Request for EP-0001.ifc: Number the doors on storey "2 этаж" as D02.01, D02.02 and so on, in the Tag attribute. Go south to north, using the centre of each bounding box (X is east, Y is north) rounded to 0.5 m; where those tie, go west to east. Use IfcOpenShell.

First a look at what the model holds.

```python
import ifcopenshell
import ifcopenshell.util.element
import ifcopenshell.util.placement

model = ifcopenshell.open("EP-0001.ifc")
print(model.schema)
storey = next(s for s in model.by_type("IfcBuildingStorey") if s.Name == "2 этаж")
doors = [e for e in ifcopenshell.util.element.get_decomposition(storey) if e.is_a("IfcDoor")]
for e in sorted(doors, key=lambda e: e.id()):
    origin = ifcopenshell.util.placement.get_local_placement(e.ObjectPlacement)[:3, 3]
    print(e.id(), e.Tag, e.Name, origin.round(2) + 0.0, sep=" | ")
```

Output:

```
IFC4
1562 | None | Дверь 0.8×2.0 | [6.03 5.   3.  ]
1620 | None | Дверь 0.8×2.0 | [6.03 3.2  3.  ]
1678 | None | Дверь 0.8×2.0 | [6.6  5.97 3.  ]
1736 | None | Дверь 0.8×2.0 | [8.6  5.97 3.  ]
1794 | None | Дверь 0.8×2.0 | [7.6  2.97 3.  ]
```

```python
import ifcopenshell
import ifcopenshell.geom
import ifcopenshell.util.element
import ifcopenshell.util.shape

model = ifcopenshell.open("EP-0001.ifc")
settings = ifcopenshell.geom.settings()
settings.set("use-world-coords", True)


def centre(element):
    shape = ifcopenshell.geom.create_shape(settings, element)
    return ifcopenshell.util.shape.get_bbox_centroid(shape.geometry)


storey = next(s for s in model.by_type("IfcBuildingStorey") if s.Name == "2 этаж")
doors = [e for e in ifcopenshell.util.element.get_decomposition(storey) if e.is_a("IfcDoor")]

# Insertion points can sit at a corner or the storey origin, so sort by the geometry (in metres).
centres = {e: centre(e) for e in doors}
doors.sort(key=lambda e: (round(centres[e][1] / 0.5), centres[e][0]))

for i, e in enumerate(doors, start=1):
    number = f"D02.{i:02d}"
    e.Tag = number
    print(e.id(), number)

model.write("EP-0001_v2.ifc")
```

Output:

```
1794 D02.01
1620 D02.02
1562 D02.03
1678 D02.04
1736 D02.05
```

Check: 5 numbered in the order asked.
